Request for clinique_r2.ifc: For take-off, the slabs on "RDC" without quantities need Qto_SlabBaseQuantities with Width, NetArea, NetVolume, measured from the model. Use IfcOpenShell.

First a look at what the model holds.

```python
import ifcopenshell
import ifcopenshell.util.element
import ifcopenshell.util.unit

model = ifcopenshell.open("clinique_r2.ifc")
print(model.schema)
for unit_type in ("LENGTHUNIT", "AREAUNIT", "VOLUMEUNIT"):
    print(unit_type, ifcopenshell.util.unit.calculate_unit_scale(model, unit_type))
storey = next(s for s in model.by_type("IfcBuildingStorey") if s.Name == "RDC")
slabs = [e for e in ifcopenshell.util.element.get_decomposition(storey) if e.is_a("IfcSlab")]
for e in sorted(slabs, key=lambda e: e.id()):
    print(e.id(), e.is_a(), e.Name, list(ifcopenshell.util.element.get_psets(e, qtos_only=True)), sep=" | ")
```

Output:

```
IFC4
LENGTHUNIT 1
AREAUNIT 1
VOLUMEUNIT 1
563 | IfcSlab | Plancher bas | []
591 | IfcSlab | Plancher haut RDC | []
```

```python
import ifcopenshell
import ifcopenshell.api.pset
import ifcopenshell.geom
import ifcopenshell.util.element
import ifcopenshell.util.shape
import ifcopenshell.util.unit

model = ifcopenshell.open("clinique_r2.ifc")
unit_scale = ifcopenshell.util.unit.calculate_unit_scale(model)
area_scale = ifcopenshell.util.unit.calculate_unit_scale(model, "AREAUNIT")
volume_scale = ifcopenshell.util.unit.calculate_unit_scale(model, "VOLUMEUNIT")
settings = ifcopenshell.geom.settings()

storey = next(s for s in model.by_type("IfcBuildingStorey") if s.Name == "RDC")
slabs = [e for e in ifcopenshell.util.element.get_decomposition(storey) if e.is_a("IfcSlab")]

for e in sorted(slabs, key=lambda e: e.id()):
    if ifcopenshell.util.element.get_psets(e, qtos_only=True, should_inherit=False):
        continue
    # Geometry comes back in metres, in the element's own axes.
    shape = ifcopenshell.geom.create_shape(settings, e)
    values = {
        "Width": ifcopenshell.util.shape.get_z(shape.geometry) / unit_scale,
        "NetArea": ifcopenshell.util.shape.get_footprint_area(shape.geometry) / area_scale,
        "NetVolume": ifcopenshell.util.shape.get_volume(shape.geometry) / volume_scale,
    }
    qto = ifcopenshell.api.pset.add_qto(model, product=e, name="Qto_SlabBaseQuantities")
    ifcopenshell.api.pset.edit_qto(model, qto=qto, properties=values)
    print(e.id(), {k: round(v, 3) for k, v in values.items()})

model.write("clinique_r2_rev.ifc")
```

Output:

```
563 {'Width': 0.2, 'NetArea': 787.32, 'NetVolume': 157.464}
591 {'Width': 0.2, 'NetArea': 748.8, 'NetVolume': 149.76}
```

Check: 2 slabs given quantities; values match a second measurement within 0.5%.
